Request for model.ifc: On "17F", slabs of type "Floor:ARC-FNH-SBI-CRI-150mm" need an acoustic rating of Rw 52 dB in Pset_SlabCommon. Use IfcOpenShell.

First a look at what the model holds.

```python
import ifcopenshell
import ifcopenshell.util.element

model = ifcopenshell.open("model.ifc")
print(model.schema)
storey = next(s for s in model.by_type("IfcBuildingStorey") if s.Name == "17F")
slabs = [e for e in ifcopenshell.util.element.get_decomposition(storey) if e.is_a("IfcSlab")]
seen = {}
for e in slabs:
    element_type = ifcopenshell.util.element.get_type(e)
    key = (element_type.Name if element_type != e and element_type else None, ifcopenshell.util.element.get_pset(e, "Pset_SlabCommon", "AcousticRating"))
    seen[key] = seen.get(key, 0) + 1
for (name, value), count in sorted(seen.items(), key=str):
    print(count, "x", name, "|", value)
```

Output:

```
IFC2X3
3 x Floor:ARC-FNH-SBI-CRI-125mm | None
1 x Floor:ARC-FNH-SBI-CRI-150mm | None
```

```python
import ifcopenshell
import ifcopenshell.api.pset
import ifcopenshell.util.element

model = ifcopenshell.open("model.ifc")

storey = next(s for s in model.by_type("IfcBuildingStorey") if s.Name == "17F")
slabs = [e for e in ifcopenshell.util.element.get_decomposition(storey) if e.is_a("IfcSlab")]

count = 0
for e in slabs:
    element_type = ifcopenshell.util.element.get_type(e)
    if element_type in (None, e) or element_type.Name != "Floor:ARC-FNH-SBI-CRI-150mm":
        continue
    # add_pset returns the element's existing set when there is one.
    pset = ifcopenshell.api.pset.add_pset(model, product=e, name="Pset_SlabCommon")
    ifcopenshell.api.pset.edit_pset(model, pset=pset, properties={"AcousticRating": "Rw 52 dB"})
    count += 1

print(count, "slabs updated")

model.write("model_updated.ifc")
```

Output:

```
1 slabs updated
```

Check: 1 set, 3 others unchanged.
